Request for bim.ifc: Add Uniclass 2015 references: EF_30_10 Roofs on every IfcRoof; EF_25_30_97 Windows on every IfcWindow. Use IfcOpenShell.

First a look at what the model holds.

```python
import ifcopenshell

model = ifcopenshell.open("bim.ifc")
print(model.schema)
print("classifications:", [c.Name for c in model.by_type("IfcClassification")])
for ifc_class in ("IfcDoor", "IfcRoof", "IfcStair", "IfcWall", "IfcWindow"):
    print(ifc_class, len(model.by_type(ifc_class)))
```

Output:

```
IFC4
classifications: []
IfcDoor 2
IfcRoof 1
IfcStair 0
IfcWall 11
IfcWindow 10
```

```python
import ifcopenshell
import ifcopenshell.api.classification

model = ifcopenshell.open("bim.ifc")

system = ifcopenshell.api.classification.add_classification(model, classification="Uniclass 2015")

codes = {
    "IfcRoof": ("EF_30_10", "Roofs"),
    "IfcWindow": ("EF_25_30_97", "Windows"),
}
for ifc_class, (code, name) in codes.items():
    products = model.by_type(ifc_class)
    ifcopenshell.api.classification.add_reference(
        model, products=products, classification=system, identification=code, name=name
    )
    print(code, len(products))

model.write("bim_updated.ifc")
```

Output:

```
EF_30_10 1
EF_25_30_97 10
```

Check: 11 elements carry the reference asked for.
